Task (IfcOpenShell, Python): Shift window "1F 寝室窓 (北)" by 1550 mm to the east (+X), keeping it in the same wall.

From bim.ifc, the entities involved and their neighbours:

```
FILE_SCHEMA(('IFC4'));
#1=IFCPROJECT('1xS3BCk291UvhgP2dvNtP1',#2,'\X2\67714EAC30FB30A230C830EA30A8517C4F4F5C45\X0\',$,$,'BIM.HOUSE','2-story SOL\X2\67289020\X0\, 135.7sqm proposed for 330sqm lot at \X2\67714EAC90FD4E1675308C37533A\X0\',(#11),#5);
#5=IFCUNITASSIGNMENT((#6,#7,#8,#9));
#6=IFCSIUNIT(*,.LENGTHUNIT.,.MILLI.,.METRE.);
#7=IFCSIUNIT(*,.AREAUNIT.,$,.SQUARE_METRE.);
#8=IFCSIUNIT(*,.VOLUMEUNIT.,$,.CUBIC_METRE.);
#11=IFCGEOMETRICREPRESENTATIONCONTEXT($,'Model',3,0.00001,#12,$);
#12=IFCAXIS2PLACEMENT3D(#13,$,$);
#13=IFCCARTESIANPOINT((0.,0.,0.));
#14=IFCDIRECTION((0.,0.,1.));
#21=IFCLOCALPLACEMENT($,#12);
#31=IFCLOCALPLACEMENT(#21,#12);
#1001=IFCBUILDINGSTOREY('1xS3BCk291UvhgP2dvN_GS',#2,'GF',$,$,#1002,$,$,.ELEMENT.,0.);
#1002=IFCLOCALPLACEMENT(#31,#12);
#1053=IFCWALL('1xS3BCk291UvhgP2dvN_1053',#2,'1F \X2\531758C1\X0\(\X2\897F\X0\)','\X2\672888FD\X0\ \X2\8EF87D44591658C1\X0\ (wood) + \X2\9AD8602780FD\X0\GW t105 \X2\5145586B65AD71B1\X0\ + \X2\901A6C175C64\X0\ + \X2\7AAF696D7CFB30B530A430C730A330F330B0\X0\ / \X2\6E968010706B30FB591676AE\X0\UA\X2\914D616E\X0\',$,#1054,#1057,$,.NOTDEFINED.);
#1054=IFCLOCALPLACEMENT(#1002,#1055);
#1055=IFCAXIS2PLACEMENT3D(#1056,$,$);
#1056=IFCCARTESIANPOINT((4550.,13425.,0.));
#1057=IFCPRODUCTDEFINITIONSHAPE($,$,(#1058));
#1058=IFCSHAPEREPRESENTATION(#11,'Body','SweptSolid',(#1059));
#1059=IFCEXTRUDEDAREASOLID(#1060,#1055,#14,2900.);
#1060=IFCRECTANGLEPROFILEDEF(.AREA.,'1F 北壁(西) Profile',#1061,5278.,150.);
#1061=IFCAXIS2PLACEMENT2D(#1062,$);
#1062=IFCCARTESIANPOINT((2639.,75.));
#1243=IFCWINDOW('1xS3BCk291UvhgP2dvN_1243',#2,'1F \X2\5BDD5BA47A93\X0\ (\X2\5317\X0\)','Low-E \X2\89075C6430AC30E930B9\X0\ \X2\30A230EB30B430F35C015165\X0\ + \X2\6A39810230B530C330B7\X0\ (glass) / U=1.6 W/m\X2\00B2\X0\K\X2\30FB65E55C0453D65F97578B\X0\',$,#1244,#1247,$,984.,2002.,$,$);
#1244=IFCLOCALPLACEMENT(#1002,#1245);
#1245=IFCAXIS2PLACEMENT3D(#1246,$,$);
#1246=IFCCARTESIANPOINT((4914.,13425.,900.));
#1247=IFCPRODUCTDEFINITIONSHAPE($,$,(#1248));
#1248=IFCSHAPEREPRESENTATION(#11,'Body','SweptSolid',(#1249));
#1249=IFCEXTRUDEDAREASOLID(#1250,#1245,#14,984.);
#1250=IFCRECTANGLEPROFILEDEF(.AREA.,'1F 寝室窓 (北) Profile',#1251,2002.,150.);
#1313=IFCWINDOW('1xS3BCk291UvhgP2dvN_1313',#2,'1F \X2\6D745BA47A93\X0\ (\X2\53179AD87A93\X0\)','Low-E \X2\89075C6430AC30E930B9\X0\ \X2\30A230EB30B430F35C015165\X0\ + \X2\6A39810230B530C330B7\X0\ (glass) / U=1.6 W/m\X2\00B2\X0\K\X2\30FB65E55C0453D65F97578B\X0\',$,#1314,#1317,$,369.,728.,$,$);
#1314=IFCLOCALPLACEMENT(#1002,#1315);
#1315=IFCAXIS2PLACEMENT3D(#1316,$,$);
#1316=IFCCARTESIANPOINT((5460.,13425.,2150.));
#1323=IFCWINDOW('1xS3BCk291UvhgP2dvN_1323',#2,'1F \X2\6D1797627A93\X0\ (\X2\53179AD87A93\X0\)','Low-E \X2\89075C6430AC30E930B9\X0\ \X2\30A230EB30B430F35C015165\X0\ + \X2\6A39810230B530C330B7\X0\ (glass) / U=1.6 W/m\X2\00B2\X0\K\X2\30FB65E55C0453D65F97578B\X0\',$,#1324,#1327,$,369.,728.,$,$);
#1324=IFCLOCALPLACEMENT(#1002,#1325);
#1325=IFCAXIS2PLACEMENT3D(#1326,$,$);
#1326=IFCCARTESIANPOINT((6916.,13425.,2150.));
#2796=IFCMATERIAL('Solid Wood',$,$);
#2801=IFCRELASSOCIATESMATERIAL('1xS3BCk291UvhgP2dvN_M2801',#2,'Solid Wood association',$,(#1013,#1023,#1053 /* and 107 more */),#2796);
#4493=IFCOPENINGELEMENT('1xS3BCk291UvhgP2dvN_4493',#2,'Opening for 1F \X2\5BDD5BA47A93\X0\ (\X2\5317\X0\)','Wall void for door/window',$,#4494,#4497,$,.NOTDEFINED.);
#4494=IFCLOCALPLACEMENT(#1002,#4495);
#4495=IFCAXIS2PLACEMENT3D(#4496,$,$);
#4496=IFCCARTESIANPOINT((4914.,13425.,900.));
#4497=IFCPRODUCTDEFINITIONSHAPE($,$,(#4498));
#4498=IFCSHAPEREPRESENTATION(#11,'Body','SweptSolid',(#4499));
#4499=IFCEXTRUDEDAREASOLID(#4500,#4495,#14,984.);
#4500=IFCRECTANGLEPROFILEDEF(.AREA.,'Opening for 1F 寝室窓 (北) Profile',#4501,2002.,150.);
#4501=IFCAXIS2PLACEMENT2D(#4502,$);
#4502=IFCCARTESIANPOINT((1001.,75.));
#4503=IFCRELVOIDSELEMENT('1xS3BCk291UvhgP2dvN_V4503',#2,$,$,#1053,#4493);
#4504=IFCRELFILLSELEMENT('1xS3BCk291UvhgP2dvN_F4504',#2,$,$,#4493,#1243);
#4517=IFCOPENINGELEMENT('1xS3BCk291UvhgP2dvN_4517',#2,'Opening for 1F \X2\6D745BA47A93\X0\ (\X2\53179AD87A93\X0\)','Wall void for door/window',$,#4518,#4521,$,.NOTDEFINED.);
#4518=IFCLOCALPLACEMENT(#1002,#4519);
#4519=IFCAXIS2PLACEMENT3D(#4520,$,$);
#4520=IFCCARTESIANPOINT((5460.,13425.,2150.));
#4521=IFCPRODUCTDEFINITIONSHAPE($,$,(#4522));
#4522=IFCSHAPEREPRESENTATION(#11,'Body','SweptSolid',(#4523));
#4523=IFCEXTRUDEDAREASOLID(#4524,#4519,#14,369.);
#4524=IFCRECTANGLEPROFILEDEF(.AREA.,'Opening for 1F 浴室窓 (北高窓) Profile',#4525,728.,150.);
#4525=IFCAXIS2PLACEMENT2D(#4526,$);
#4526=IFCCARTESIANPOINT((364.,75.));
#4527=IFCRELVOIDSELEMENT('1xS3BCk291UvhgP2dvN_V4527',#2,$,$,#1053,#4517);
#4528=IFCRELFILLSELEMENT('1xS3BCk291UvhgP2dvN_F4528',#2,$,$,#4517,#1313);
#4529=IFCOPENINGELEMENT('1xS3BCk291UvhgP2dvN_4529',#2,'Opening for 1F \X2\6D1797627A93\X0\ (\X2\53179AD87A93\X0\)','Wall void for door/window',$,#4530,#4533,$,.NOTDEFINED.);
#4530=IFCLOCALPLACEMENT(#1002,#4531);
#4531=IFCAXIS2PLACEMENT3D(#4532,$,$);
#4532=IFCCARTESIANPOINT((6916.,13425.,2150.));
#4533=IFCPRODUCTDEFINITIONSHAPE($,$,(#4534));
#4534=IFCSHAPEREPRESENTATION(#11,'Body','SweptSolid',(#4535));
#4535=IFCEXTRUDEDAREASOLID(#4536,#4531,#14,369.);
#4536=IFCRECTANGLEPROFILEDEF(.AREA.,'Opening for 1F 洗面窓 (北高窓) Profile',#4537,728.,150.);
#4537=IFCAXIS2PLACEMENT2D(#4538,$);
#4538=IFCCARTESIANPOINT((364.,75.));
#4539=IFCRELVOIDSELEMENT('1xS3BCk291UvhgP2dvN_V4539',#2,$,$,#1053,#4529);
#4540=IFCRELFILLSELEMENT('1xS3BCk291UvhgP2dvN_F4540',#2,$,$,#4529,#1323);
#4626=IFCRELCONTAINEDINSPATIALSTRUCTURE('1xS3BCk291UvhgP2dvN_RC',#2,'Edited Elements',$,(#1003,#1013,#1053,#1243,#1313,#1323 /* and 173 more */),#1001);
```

```python
import ifcopenshell
import ifcopenshell.api.geometry
import ifcopenshell.util.placement

model = ifcopenshell.open("bim.ifc")

window = model.by_guid("1xS3BCk291UvhgP2dvN_1243")
opening = window.FillsVoids[0].RelatingOpeningElement
wall = opening.VoidsElements[0].RelatingBuildingElement

wall_matrix = ifcopenshell.util.placement.get_local_placement(wall.ObjectPlacement)
shift = wall_matrix[:3, 0] * 1550.0
before = ifcopenshell.util.placement.get_local_placement(window.ObjectPlacement)[:3, 3].copy()

# The window is not placed relative to its opening, so move both.
for product in (opening, window):
    matrix = ifcopenshell.util.placement.get_local_placement(product.ObjectPlacement)
    matrix[:3, 3] += shift
    ifcopenshell.api.geometry.edit_object_placement(model, product=product, matrix=matrix, is_si=False)

after = ifcopenshell.util.placement.get_local_placement(window.ObjectPlacement)[:3, 3]
print("window moved by", (after - before).round(3) + 0.0)

model.write("bim_rev.ifc")
```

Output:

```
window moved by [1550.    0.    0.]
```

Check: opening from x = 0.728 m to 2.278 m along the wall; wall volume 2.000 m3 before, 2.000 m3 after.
